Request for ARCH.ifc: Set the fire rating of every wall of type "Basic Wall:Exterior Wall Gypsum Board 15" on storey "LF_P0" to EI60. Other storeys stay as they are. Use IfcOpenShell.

First a look at what the model holds.

```python
import ifcopenshell
import ifcopenshell.util.element

model = ifcopenshell.open("ARCH.ifc")
print(model.schema)
storey = next(s for s in model.by_type("IfcBuildingStorey") if s.Name == "LF_P0")
walls = [e for e in ifcopenshell.util.element.get_decomposition(storey) if e.is_a("IfcWall")]
seen = {}
for e in walls:
    element_type = ifcopenshell.util.element.get_type(e)
    key = (element_type.Name if element_type != e and element_type else None, ifcopenshell.util.element.get_pset(e, "Pset_WallCommon", "FireRating"))
    seen[key] = seen.get(key, 0) + 1
for (name, value), count in sorted(seen.items(), key=str):
    print(count, "x", name, "|", value)
```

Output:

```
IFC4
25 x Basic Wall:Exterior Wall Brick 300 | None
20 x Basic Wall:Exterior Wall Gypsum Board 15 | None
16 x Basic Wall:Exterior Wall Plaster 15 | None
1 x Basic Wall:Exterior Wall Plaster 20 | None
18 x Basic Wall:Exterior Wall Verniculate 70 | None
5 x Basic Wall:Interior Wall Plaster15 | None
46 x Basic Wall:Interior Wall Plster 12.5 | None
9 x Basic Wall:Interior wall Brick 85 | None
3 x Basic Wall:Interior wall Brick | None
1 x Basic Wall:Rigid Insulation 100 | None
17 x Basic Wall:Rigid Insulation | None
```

```python
import ifcopenshell
import ifcopenshell.api.pset
import ifcopenshell.util.element

model = ifcopenshell.open("ARCH.ifc")

storey = next(s for s in model.by_type("IfcBuildingStorey") if s.Name == "LF_P0")
walls = [e for e in ifcopenshell.util.element.get_decomposition(storey) if e.is_a("IfcWall")]

count = 0
for e in walls:
    element_type = ifcopenshell.util.element.get_type(e)
    if element_type in (None, e) or element_type.Name != "Basic Wall:Exterior Wall Gypsum Board 15":
        continue
    # add_pset returns the element's existing set when there is one.
    pset = ifcopenshell.api.pset.add_pset(model, product=e, name="Pset_WallCommon")
    ifcopenshell.api.pset.edit_pset(model, pset=pset, properties={"FireRating": "EI60"})
    count += 1

print(count, "walls updated")

model.write("ARCH_v2.ifc")
```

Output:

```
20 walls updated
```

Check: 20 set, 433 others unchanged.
